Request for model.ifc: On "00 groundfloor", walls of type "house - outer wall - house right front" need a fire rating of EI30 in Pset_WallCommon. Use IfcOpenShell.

First a look at what the model holds.

```python
import ifcopenshell
import ifcopenshell.util.element

model = ifcopenshell.open("model.ifc")
print(model.schema)
storey = next(s for s in model.by_type("IfcBuildingStorey") if s.Name == "00 groundfloor")
walls = [e for e in ifcopenshell.util.element.get_decomposition(storey) if e.is_a("IfcWall")]
seen = {}
for e in walls:
    element_type = ifcopenshell.util.element.get_type(e)
    key = (element_type.Name if element_type != e and element_type else None, ifcopenshell.util.element.get_pset(e, "Pset_WallCommon", "FireRating"))
    seen[key] = seen.get(key, 0) + 1
for (name, value), count in sorted(seen.items(), key=str):
    print(count, "x", name, "|", value)
```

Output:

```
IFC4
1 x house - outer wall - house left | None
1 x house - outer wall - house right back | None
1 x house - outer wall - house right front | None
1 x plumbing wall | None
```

```python
import ifcopenshell
import ifcopenshell.api.pset
import ifcopenshell.util.element

model = ifcopenshell.open("model.ifc")

storey = next(s for s in model.by_type("IfcBuildingStorey") if s.Name == "00 groundfloor")
walls = [e for e in ifcopenshell.util.element.get_decomposition(storey) if e.is_a("IfcWall")]

count = 0
for e in walls:
    element_type = ifcopenshell.util.element.get_type(e)
    if element_type in (None, e) or element_type.Name != "house - outer wall - house right front":
        continue
    # add_pset returns the element's existing set when there is one.
    pset = ifcopenshell.api.pset.add_pset(model, product=e, name="Pset_WallCommon")
    ifcopenshell.api.pset.edit_pset(model, pset=pset, properties={"FireRating": "EI30"})
    count += 1

print(count, "walls updated")

model.write("model_v2.ifc")
```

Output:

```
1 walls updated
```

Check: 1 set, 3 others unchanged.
